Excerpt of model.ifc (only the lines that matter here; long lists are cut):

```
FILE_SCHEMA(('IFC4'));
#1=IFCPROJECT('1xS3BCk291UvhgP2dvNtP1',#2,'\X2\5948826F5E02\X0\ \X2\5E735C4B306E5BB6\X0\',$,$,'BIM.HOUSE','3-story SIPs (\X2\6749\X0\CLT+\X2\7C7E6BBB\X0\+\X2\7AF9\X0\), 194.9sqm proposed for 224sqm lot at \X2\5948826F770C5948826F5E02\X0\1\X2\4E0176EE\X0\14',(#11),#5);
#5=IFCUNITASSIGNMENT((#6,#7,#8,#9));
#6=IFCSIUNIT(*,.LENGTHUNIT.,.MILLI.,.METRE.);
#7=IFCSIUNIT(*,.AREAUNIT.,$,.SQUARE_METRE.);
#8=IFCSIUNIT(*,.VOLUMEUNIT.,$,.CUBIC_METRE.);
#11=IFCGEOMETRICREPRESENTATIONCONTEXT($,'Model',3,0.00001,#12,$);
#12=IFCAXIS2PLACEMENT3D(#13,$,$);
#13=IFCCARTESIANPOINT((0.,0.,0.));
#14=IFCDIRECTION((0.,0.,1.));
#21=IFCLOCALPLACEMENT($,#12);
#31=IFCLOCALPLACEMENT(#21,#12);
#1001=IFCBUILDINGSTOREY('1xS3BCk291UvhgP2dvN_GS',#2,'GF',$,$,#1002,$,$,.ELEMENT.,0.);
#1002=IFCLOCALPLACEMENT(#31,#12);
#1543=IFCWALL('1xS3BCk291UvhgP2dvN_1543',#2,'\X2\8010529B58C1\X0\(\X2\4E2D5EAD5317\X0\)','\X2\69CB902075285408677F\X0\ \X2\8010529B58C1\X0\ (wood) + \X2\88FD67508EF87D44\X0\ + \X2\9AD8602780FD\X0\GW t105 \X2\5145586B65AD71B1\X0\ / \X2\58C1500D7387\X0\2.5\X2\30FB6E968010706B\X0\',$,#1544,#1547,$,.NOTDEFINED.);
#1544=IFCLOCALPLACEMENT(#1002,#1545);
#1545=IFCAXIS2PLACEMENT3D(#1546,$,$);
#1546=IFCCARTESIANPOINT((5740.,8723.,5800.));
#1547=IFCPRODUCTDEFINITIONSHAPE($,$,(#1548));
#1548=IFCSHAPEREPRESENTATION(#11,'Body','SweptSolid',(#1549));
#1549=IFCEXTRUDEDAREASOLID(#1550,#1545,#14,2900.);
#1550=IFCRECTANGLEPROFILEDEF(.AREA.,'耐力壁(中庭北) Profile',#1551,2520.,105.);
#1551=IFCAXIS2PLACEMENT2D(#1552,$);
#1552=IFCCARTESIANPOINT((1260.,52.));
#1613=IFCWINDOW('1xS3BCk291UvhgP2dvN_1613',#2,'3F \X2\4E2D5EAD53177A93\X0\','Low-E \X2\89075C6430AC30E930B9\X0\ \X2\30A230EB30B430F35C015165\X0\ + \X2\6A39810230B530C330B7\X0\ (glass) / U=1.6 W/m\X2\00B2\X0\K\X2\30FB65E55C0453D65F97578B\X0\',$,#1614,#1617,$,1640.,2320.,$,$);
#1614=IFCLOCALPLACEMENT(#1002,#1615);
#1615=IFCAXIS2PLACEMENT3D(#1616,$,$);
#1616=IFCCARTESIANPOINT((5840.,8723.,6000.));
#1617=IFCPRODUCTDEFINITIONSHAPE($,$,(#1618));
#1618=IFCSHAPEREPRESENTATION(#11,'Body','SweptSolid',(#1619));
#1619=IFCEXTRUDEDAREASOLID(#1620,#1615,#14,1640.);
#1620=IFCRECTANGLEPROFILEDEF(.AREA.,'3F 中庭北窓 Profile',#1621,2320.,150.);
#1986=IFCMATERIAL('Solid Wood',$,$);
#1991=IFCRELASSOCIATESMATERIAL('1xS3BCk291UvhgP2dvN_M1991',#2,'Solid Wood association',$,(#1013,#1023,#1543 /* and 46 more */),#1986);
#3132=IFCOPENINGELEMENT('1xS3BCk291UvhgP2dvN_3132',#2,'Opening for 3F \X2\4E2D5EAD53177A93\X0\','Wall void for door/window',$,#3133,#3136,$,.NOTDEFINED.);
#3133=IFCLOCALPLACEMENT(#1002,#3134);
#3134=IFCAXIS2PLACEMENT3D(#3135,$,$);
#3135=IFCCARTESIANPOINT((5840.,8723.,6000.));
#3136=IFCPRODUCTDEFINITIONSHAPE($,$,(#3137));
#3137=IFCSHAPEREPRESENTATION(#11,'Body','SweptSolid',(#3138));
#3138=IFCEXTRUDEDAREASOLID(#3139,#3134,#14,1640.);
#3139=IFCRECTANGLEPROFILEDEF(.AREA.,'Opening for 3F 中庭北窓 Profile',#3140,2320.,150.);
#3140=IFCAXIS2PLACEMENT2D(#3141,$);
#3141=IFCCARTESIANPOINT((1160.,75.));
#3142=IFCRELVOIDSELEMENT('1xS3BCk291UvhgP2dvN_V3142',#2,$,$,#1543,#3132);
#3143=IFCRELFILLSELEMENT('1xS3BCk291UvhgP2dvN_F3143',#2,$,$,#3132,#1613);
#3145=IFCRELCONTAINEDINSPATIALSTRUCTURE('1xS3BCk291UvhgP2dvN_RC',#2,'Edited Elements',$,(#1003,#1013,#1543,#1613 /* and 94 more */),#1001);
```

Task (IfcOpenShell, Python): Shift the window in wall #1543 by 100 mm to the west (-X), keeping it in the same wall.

```python
import ifcopenshell
import ifcopenshell.api.geometry
import ifcopenshell.util.placement

model = ifcopenshell.open("model.ifc")

window = model.by_guid("1xS3BCk291UvhgP2dvN_1613")
opening = window.FillsVoids[0].RelatingOpeningElement
wall = opening.VoidsElements[0].RelatingBuildingElement

wall_matrix = ifcopenshell.util.placement.get_local_placement(wall.ObjectPlacement)
shift = wall_matrix[:3, 0] * -100.0
before = ifcopenshell.util.placement.get_local_placement(window.ObjectPlacement)[:3, 3].copy()

# The window is not placed relative to its opening, so move both.
for product in (opening, window):
    matrix = ifcopenshell.util.placement.get_local_placement(product.ObjectPlacement)
    matrix[:3, 3] += shift
    ifcopenshell.api.geometry.edit_object_placement(model, product=product, matrix=matrix, is_si=False)

after = ifcopenshell.util.placement.get_local_placement(window.ObjectPlacement)[:3, 3]
print("window moved by", (after - before).round(3) + 0.0)

model.write("model_v2.ifc")
```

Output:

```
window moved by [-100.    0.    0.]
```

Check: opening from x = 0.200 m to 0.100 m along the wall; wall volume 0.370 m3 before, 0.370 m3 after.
